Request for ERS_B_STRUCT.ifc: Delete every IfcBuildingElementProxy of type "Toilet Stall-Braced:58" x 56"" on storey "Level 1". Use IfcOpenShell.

First a look at what the model holds.

```python
import ifcopenshell
import ifcopenshell.util.element

model = ifcopenshell.open("ERS_B_STRUCT.ifc")
print(model.schema)
storey = next(s for s in model.by_type("IfcBuildingStorey") if s.Name == "Level 1")
proxies = [e for e in ifcopenshell.util.element.get_decomposition(storey) if e.is_a("IfcBuildingElementProxy")]
seen = {}
for e in proxies:
    element_type = ifcopenshell.util.element.get_type(e)
    name = element_type.Name if element_type not in (None, e) else None
    seen[name] = seen.get(name, 0) + 1
for name, count in sorted(seen.items(), key=str):
    print(count, "x", name)
```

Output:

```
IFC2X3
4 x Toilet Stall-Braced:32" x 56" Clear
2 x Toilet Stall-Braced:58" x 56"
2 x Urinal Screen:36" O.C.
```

```python
import ifcopenshell
import ifcopenshell.api.root
import ifcopenshell.util.element

model = ifcopenshell.open("ERS_B_STRUCT.ifc")

storey = next(s for s in model.by_type("IfcBuildingStorey") if s.Name == "Level 1")
proxies = [e for e in ifcopenshell.util.element.get_decomposition(storey) if e.is_a("IfcBuildingElementProxy")]
targets = [e for e in proxies if (t := ifcopenshell.util.element.get_type(e)) not in (None, e) and t.Name == 'Toilet Stall-Braced:58" x 56"']

for e in targets:
    ifcopenshell.api.root.remove_product(model, product=e)
print(len(targets), "removed")

model.write("ERS_B_STRUCT-out.ifc")
```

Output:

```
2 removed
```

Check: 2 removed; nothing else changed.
